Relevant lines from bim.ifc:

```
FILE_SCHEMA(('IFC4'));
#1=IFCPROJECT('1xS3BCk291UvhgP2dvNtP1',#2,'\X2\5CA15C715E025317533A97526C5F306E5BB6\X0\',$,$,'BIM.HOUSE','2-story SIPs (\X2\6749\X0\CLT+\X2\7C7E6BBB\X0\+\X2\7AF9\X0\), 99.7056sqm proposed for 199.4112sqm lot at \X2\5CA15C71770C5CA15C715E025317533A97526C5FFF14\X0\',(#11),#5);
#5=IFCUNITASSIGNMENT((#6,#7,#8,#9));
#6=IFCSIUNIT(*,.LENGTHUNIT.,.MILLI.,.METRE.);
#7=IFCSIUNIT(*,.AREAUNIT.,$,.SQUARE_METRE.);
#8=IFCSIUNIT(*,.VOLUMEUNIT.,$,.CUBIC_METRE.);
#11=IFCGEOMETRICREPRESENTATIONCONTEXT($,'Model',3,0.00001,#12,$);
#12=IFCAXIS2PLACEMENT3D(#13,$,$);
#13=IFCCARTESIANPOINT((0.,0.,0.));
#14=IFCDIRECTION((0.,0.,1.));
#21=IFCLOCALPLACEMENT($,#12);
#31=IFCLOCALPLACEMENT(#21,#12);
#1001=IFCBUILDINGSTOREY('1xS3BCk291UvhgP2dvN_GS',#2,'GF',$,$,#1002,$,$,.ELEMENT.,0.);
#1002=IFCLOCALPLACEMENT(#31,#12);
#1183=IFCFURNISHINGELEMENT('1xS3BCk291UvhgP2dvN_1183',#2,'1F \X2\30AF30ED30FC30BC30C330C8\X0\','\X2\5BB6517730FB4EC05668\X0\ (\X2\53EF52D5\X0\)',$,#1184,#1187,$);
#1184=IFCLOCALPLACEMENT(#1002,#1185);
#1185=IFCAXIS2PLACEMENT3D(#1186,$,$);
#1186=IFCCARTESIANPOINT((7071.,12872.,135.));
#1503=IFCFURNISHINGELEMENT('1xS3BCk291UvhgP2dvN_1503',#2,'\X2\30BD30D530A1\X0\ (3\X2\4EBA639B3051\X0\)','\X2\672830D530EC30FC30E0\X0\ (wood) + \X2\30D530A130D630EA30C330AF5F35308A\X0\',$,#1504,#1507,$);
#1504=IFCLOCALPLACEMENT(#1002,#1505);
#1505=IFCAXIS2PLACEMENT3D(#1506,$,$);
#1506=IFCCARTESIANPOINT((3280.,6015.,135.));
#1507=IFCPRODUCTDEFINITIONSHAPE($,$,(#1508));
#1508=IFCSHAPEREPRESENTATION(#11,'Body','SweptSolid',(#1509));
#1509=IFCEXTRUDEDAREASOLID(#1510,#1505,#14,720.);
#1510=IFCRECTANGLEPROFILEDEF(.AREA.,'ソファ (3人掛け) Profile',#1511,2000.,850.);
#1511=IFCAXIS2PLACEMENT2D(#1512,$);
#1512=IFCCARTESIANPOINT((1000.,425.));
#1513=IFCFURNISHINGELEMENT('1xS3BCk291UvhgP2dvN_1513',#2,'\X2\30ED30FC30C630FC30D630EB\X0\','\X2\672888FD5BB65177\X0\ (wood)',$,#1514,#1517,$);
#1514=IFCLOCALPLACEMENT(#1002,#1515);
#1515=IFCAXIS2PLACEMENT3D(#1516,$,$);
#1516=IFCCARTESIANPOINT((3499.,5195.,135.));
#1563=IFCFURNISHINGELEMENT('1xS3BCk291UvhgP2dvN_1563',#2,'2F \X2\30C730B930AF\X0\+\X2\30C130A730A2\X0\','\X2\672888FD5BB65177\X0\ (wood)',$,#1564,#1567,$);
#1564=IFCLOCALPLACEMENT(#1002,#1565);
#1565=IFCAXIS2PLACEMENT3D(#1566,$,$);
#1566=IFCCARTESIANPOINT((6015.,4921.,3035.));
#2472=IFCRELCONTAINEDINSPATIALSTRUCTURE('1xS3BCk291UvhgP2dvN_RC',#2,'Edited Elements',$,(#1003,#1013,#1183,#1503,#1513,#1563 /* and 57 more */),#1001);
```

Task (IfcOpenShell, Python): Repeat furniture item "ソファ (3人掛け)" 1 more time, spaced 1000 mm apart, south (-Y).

```python
import numpy as np
import ifcopenshell
import ifcopenshell.api.geometry
import ifcopenshell.api.root
import ifcopenshell.util.element
import ifcopenshell.util.placement
import ifcopenshell.util.unit

model = ifcopenshell.open("bim.ifc")
unit_scale = ifcopenshell.util.unit.calculate_unit_scale(model)


def reuse_history(source, copy):
    """copy_class also copies each property set's owner history, people and application; keep the originals."""
    for rel in copy.IsDefinedBy:
        if rel.is_a("IfcRelDefinesByProperties") and (history := rel.RelatingPropertyDefinition.OwnerHistory):
            rel.RelatingPropertyDefinition.OwnerHistory = source.OwnerHistory
            ifcopenshell.util.element.remove_deep2(model, history)


source = model.by_guid("1xS3BCk291UvhgP2dvN_1503")
base = ifcopenshell.util.placement.get_local_placement(source.ObjectPlacement)
step = np.array([0.0, -1.0, 0.0]) * 1 / unit_scale

for i in range(1, 2):
    copy = ifcopenshell.api.root.copy_class(model, product=source)
    copy.Representation = ifcopenshell.util.element.copy_deep(
        model, source.Representation, exclude=["IfcGeometricRepresentationContext", "IfcRepresentationMap"]
    )
    reuse_history(source, copy)
    matrix = base.copy()
    matrix[:3, 3] += i * step
    print("added at", matrix[:3, 3].round(3) + 0.0)
    ifcopenshell.api.geometry.edit_object_placement(model, product=copy, matrix=matrix, is_si=False)

model.write("bim_edited.ifc")
```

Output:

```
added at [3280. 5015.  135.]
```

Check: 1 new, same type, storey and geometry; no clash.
